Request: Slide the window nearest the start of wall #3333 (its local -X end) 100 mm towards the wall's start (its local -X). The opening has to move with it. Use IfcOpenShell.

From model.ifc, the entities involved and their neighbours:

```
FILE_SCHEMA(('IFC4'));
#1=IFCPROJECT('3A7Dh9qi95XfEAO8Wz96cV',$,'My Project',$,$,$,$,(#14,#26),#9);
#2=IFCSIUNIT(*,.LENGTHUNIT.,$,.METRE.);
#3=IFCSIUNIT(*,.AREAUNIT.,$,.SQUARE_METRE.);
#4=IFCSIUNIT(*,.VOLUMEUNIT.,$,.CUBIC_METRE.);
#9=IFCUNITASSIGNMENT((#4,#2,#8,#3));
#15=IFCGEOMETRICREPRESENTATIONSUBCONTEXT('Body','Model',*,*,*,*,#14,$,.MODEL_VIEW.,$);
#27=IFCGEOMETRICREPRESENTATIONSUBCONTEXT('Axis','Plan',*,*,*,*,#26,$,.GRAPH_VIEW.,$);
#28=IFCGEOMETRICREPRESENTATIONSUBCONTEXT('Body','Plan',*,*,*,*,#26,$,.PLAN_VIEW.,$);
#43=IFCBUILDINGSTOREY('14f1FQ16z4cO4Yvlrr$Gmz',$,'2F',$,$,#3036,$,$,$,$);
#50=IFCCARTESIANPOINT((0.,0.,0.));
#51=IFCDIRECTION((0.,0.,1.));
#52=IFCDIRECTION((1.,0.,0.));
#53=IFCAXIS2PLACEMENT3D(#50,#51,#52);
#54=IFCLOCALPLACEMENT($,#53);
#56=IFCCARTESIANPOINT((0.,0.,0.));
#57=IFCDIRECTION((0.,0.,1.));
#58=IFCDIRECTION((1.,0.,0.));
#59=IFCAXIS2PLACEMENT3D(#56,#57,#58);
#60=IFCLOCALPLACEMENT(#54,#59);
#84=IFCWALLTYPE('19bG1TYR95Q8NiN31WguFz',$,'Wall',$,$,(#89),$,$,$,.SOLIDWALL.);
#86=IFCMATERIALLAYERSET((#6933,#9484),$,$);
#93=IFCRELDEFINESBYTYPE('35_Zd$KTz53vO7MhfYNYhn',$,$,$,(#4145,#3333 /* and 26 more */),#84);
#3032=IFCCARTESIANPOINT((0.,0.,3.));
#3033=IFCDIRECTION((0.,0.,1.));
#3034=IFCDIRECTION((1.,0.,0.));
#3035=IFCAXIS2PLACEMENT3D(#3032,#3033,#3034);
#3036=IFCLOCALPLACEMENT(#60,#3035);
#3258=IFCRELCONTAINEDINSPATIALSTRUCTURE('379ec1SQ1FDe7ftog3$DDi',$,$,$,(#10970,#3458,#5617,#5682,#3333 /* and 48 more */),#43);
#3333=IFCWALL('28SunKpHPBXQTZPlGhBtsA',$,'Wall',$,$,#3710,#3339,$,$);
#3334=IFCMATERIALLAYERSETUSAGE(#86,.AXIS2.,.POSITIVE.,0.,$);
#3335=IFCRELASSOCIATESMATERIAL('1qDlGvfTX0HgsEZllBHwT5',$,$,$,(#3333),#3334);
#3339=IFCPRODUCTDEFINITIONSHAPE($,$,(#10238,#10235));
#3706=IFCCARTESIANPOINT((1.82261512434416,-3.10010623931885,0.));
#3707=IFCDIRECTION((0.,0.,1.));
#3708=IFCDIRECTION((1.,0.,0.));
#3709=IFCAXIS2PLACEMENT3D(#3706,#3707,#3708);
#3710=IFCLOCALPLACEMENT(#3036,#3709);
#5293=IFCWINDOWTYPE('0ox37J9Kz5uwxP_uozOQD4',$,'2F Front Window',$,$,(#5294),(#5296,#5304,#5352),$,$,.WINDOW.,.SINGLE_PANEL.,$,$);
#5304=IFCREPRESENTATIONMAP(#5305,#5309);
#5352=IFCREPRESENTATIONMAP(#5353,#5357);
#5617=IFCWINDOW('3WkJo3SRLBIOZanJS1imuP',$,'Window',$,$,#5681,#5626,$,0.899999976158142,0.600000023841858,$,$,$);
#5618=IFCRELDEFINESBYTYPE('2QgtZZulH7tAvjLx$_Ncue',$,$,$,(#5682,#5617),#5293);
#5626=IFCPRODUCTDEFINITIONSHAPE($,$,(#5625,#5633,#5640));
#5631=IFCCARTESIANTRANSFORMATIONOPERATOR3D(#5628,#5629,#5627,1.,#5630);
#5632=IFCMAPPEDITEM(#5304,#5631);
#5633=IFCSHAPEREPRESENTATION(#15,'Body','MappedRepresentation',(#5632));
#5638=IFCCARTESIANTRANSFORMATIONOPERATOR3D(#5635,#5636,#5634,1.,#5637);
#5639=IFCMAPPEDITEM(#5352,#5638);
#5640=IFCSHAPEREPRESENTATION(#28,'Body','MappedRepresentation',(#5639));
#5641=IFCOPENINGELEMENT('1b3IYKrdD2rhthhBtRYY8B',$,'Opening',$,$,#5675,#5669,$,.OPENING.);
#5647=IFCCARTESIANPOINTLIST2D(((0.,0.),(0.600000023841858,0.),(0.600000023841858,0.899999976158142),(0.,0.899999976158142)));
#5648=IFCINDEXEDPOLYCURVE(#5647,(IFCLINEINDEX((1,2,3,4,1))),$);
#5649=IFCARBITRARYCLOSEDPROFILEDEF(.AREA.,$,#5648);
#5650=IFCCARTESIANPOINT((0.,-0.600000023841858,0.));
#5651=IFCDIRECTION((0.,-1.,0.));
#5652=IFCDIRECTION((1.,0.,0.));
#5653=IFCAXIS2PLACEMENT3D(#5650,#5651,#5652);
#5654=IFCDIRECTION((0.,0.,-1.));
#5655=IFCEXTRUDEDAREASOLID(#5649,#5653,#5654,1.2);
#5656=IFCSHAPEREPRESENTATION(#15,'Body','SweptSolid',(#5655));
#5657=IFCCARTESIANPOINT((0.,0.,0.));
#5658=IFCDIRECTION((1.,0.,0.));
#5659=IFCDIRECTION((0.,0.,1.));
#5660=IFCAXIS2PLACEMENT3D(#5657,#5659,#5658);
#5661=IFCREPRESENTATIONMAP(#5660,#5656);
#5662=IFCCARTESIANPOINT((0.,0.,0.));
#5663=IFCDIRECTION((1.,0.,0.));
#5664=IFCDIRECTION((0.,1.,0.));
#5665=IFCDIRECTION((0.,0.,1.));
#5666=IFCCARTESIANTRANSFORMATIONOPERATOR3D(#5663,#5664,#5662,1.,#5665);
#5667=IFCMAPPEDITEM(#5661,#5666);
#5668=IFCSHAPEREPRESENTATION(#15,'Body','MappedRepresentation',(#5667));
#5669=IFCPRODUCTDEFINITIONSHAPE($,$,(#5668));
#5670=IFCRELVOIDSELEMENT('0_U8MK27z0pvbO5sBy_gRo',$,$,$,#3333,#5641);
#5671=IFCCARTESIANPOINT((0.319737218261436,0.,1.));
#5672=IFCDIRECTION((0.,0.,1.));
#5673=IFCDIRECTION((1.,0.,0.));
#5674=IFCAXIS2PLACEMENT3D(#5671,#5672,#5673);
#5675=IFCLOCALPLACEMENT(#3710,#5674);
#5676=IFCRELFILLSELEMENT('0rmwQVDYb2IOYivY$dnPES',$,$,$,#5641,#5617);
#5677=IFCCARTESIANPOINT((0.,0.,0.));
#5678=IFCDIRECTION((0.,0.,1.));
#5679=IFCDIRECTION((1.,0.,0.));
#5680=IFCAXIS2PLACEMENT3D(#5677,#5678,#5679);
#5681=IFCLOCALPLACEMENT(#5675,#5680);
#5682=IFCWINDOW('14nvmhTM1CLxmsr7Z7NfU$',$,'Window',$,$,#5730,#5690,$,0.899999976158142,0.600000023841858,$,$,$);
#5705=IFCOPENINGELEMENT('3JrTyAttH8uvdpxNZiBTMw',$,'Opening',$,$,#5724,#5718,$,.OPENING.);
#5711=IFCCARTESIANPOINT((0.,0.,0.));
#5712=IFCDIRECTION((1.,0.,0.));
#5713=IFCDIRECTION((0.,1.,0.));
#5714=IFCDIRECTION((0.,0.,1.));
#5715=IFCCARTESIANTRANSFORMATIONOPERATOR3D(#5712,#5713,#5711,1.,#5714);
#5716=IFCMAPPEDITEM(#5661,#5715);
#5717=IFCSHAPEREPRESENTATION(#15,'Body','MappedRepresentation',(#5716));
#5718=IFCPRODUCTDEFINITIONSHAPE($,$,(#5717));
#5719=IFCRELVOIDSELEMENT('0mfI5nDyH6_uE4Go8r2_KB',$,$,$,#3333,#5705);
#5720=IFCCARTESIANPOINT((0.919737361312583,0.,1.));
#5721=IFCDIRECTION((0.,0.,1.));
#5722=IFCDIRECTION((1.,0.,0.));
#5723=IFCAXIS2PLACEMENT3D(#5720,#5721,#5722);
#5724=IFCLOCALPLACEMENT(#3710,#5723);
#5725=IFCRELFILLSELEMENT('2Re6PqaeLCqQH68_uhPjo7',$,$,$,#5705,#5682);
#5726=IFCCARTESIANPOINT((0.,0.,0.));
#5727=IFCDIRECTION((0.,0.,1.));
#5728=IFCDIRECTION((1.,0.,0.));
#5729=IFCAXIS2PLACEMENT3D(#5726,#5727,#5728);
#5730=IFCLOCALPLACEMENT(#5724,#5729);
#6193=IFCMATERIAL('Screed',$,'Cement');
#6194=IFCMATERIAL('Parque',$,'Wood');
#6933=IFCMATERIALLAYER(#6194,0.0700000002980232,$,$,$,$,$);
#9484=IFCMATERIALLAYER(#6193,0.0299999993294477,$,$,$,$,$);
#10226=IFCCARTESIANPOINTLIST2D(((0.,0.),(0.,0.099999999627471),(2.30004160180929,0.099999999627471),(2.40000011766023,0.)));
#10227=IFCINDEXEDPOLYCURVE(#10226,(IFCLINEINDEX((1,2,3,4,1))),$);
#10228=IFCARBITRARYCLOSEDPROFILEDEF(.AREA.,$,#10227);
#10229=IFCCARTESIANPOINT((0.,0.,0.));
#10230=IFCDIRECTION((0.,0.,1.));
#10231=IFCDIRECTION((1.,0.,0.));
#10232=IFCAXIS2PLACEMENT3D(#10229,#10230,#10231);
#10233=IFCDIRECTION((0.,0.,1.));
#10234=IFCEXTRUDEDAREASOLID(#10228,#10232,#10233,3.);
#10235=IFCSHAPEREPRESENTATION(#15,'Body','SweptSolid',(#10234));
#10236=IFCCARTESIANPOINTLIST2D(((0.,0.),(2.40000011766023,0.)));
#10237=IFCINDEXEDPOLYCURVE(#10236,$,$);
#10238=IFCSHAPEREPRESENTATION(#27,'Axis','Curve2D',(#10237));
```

```python
import ifcopenshell
import ifcopenshell.api.geometry
import ifcopenshell.util.placement
import ifcopenshell.util.unit

model = ifcopenshell.open("model.ifc")
unit_scale = ifcopenshell.util.unit.calculate_unit_scale(model)

window = model.by_id(5617)
opening = window.FillsVoids[0].RelatingOpeningElement
wall = opening.VoidsElements[0].RelatingBuildingElement

wall_matrix = ifcopenshell.util.placement.get_local_placement(wall.ObjectPlacement)
shift = wall_matrix[:3, 0] * -0.1 / unit_scale
before = ifcopenshell.util.placement.get_local_placement(window.ObjectPlacement)[:3, 3].copy()

# The window is placed relative to its opening, so it follows when the opening moves.
matrix = ifcopenshell.util.placement.get_local_placement(opening.ObjectPlacement)
matrix[:3, 3] += shift
ifcopenshell.api.geometry.edit_object_placement(
    model, product=opening, matrix=matrix, is_si=False, should_transform_children=True
)

after = ifcopenshell.util.placement.get_local_placement(window.ObjectPlacement)[:3, 3]
print("window moved by", (after - before).round(3) + 0.0)

model.write("model-out.ifc")
```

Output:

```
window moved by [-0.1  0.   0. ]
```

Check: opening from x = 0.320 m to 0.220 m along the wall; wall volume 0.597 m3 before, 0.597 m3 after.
